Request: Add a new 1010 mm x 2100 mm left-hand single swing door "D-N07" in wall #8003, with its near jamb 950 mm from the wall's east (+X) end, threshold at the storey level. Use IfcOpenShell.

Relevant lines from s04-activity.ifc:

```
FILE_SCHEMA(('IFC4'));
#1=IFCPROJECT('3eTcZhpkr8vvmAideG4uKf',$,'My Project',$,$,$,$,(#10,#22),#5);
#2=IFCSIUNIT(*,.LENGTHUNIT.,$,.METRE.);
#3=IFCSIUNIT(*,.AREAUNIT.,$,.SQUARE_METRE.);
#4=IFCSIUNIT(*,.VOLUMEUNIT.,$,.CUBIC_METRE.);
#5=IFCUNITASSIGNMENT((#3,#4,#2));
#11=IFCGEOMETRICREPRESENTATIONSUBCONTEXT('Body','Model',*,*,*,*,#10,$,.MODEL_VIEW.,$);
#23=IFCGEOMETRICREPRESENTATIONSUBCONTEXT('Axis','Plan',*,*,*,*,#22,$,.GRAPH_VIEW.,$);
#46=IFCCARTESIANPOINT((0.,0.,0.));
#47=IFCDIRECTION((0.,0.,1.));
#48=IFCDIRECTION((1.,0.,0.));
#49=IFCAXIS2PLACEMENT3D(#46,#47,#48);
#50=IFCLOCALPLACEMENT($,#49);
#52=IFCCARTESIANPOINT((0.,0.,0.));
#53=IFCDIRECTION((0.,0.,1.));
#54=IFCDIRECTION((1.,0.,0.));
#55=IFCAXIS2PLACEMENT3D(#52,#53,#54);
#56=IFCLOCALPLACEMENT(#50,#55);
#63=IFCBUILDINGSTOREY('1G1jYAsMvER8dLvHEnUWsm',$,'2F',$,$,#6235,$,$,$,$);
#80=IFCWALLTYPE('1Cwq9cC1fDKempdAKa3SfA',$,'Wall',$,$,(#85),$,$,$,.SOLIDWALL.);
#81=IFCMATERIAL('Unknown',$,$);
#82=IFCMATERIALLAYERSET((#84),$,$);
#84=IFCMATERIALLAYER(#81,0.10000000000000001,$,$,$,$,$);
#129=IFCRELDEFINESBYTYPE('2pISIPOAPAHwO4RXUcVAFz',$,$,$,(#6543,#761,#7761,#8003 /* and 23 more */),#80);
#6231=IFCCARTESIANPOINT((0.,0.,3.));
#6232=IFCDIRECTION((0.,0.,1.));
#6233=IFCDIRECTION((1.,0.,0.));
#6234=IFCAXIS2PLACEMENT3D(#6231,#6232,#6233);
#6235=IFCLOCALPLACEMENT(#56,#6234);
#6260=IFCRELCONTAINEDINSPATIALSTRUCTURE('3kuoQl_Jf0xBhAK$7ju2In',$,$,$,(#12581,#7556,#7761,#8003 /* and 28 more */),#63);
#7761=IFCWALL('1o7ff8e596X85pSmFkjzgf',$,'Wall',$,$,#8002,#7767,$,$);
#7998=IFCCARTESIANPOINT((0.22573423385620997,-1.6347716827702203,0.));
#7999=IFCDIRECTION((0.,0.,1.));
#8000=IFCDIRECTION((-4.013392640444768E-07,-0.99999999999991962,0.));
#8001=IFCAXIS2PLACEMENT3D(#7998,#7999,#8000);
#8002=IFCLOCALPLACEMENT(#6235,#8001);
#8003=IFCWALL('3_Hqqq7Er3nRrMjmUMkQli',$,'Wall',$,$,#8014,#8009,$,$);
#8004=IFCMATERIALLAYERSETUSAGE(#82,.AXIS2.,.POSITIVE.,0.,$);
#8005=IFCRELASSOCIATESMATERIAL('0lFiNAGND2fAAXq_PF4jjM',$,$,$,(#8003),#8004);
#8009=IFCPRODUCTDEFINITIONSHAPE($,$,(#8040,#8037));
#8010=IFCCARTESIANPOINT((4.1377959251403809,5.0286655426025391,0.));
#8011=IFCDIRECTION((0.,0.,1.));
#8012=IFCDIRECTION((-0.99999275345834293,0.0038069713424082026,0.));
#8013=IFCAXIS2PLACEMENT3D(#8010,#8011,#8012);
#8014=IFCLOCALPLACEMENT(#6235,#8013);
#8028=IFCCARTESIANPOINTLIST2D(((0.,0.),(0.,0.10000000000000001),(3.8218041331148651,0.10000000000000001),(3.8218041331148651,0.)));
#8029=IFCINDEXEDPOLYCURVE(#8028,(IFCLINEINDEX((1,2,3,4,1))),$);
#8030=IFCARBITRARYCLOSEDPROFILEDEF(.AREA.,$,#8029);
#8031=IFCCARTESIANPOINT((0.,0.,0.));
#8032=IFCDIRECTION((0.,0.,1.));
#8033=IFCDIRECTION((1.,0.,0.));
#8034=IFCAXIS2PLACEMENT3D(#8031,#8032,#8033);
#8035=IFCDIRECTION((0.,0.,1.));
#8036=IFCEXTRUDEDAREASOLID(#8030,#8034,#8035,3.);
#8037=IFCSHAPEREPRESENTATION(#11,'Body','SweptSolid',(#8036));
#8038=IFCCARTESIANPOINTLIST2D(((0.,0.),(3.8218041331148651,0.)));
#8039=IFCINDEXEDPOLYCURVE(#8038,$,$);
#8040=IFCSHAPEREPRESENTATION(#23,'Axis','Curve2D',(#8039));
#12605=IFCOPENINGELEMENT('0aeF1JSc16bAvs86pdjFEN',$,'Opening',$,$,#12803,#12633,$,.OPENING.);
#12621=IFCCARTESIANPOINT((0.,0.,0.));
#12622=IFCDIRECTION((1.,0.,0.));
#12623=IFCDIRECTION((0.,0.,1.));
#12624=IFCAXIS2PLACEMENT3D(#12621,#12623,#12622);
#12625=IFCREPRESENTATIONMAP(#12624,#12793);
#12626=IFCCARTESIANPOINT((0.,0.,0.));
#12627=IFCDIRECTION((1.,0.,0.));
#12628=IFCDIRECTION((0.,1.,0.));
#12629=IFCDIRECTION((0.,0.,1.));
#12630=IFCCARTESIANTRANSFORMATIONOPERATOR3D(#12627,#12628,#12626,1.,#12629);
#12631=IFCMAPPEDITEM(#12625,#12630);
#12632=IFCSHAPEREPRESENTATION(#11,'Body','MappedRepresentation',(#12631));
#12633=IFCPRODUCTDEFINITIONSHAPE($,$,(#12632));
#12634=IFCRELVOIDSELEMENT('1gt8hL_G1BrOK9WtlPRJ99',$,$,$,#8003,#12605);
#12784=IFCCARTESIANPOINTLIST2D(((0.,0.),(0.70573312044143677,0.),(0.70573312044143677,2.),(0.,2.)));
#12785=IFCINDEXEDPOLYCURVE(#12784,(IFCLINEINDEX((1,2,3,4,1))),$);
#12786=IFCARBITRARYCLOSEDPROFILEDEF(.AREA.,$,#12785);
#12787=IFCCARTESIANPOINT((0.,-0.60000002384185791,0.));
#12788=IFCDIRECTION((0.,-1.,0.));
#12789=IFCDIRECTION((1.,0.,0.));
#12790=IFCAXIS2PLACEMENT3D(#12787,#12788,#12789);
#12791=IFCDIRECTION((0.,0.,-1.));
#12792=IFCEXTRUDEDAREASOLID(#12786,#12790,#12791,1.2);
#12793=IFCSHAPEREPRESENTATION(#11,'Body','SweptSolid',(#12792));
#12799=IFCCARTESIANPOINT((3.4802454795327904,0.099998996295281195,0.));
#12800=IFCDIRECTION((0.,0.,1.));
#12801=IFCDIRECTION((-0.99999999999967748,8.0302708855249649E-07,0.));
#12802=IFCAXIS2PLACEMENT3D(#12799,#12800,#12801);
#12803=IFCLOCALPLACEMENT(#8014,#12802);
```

```python
import numpy as np
import ifcopenshell
import ifcopenshell.api.feature
import ifcopenshell.api.geometry
import ifcopenshell.api.root
import ifcopenshell.api.spatial
import ifcopenshell.geom
import ifcopenshell.util.element
import ifcopenshell.util.placement
import ifcopenshell.util.representation
import ifcopenshell.util.shape
import ifcopenshell.util.unit

model = ifcopenshell.open("s04-activity.ifc")
unit_scale = ifcopenshell.util.unit.calculate_unit_scale(model)
settings = ifcopenshell.geom.settings()


def volume(element):
    """Net volume in cubic metres, openings subtracted."""
    shape = ifcopenshell.geom.create_shape(settings, element)
    return ifcopenshell.util.shape.get_volume(shape.geometry)


wall = model.by_guid("3_Hqqq7Er3nRrMjmUMkQli")
storey = ifcopenshell.util.element.get_container(wall, ifc_class="IfcBuildingStorey")
context = ifcopenshell.util.representation.get_context(model, "Model", "Body", "MODEL_VIEW")
before = volume(wall)

width, height, from_end, sill = 1.01, 2.1, 0.95, 0.0  # metres

# The wall runs along its own X axis, and the end named is its -X end.
wall_shape = ifcopenshell.geom.create_shape(settings, wall)
x, y, z = ifcopenshell.util.shape.get_vertices(wall_shape.geometry).T
start = x.min() + from_end
face, thickness = float(y.min()), float(y.max() - y.min())
wall_matrix = ifcopenshell.util.placement.get_local_placement(wall.ObjectPlacement)
level = ifcopenshell.util.placement.get_local_placement(storey.ObjectPlacement)[2, 3]


def in_wall(x, y):
    """Placement at x, y metres in the wall's axes, at sill height."""
    matrix = wall_matrix.copy()
    matrix[:, 3] = wall_matrix @ np.array([x / unit_scale, y / unit_scale, 0.0, 1.0])
    matrix[2, 3] = level + sill / unit_scale
    return matrix


# Opening: a box that overshoots both wall faces by 50 mm.
opening = ifcopenshell.api.root.create_entity(model, ifc_class="IfcOpeningElement", predefined_type="OPENING")
box = ifcopenshell.api.geometry.add_wall_representation(
    model, context=context, length=width, height=height, thickness=thickness + 0.1
)
ifcopenshell.api.geometry.assign_representation(model, product=opening, representation=box)
ifcopenshell.api.geometry.edit_object_placement(model, product=opening, matrix=in_wall(start, face - 0.05), is_si=False)
ifcopenshell.api.feature.add_feature(model, feature=opening, element=wall)

door = ifcopenshell.api.root.create_entity(model, ifc_class="IfcDoor", name="D-N07", predefined_type="DOOR")
door.OverallWidth, door.OverallHeight = width / unit_scale, height / unit_scale
door.OperationType = "SINGLE_SWING_LEFT"
body = ifcopenshell.api.geometry.add_door_representation(
    model,
    context=context,
    overall_width=door.OverallWidth,
    overall_height=door.OverallHeight,
    operation_type="SINGLE_SWING_LEFT",
    lining_properties={"LiningDepth": thickness / unit_scale, "ThresholdDepth": thickness / unit_scale},
)
ifcopenshell.api.geometry.assign_representation(model, product=door, representation=body)
ifcopenshell.api.spatial.assign_container(model, products=[door], relating_structure=storey)
ifcopenshell.api.feature.add_filling(model, opening=opening, element=door)

# The lining spans the wall, so the door starts at the wall face.
ifcopenshell.api.geometry.edit_object_placement(model, product=door, matrix=in_wall(start, face), is_si=False)

after = volume(wall)

print(f"wall volume {before:.3f} -> {after:.3f} m3")

model.write("s04-activity_rev.ifc")
```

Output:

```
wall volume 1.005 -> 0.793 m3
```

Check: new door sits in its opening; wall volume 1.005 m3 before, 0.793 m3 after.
